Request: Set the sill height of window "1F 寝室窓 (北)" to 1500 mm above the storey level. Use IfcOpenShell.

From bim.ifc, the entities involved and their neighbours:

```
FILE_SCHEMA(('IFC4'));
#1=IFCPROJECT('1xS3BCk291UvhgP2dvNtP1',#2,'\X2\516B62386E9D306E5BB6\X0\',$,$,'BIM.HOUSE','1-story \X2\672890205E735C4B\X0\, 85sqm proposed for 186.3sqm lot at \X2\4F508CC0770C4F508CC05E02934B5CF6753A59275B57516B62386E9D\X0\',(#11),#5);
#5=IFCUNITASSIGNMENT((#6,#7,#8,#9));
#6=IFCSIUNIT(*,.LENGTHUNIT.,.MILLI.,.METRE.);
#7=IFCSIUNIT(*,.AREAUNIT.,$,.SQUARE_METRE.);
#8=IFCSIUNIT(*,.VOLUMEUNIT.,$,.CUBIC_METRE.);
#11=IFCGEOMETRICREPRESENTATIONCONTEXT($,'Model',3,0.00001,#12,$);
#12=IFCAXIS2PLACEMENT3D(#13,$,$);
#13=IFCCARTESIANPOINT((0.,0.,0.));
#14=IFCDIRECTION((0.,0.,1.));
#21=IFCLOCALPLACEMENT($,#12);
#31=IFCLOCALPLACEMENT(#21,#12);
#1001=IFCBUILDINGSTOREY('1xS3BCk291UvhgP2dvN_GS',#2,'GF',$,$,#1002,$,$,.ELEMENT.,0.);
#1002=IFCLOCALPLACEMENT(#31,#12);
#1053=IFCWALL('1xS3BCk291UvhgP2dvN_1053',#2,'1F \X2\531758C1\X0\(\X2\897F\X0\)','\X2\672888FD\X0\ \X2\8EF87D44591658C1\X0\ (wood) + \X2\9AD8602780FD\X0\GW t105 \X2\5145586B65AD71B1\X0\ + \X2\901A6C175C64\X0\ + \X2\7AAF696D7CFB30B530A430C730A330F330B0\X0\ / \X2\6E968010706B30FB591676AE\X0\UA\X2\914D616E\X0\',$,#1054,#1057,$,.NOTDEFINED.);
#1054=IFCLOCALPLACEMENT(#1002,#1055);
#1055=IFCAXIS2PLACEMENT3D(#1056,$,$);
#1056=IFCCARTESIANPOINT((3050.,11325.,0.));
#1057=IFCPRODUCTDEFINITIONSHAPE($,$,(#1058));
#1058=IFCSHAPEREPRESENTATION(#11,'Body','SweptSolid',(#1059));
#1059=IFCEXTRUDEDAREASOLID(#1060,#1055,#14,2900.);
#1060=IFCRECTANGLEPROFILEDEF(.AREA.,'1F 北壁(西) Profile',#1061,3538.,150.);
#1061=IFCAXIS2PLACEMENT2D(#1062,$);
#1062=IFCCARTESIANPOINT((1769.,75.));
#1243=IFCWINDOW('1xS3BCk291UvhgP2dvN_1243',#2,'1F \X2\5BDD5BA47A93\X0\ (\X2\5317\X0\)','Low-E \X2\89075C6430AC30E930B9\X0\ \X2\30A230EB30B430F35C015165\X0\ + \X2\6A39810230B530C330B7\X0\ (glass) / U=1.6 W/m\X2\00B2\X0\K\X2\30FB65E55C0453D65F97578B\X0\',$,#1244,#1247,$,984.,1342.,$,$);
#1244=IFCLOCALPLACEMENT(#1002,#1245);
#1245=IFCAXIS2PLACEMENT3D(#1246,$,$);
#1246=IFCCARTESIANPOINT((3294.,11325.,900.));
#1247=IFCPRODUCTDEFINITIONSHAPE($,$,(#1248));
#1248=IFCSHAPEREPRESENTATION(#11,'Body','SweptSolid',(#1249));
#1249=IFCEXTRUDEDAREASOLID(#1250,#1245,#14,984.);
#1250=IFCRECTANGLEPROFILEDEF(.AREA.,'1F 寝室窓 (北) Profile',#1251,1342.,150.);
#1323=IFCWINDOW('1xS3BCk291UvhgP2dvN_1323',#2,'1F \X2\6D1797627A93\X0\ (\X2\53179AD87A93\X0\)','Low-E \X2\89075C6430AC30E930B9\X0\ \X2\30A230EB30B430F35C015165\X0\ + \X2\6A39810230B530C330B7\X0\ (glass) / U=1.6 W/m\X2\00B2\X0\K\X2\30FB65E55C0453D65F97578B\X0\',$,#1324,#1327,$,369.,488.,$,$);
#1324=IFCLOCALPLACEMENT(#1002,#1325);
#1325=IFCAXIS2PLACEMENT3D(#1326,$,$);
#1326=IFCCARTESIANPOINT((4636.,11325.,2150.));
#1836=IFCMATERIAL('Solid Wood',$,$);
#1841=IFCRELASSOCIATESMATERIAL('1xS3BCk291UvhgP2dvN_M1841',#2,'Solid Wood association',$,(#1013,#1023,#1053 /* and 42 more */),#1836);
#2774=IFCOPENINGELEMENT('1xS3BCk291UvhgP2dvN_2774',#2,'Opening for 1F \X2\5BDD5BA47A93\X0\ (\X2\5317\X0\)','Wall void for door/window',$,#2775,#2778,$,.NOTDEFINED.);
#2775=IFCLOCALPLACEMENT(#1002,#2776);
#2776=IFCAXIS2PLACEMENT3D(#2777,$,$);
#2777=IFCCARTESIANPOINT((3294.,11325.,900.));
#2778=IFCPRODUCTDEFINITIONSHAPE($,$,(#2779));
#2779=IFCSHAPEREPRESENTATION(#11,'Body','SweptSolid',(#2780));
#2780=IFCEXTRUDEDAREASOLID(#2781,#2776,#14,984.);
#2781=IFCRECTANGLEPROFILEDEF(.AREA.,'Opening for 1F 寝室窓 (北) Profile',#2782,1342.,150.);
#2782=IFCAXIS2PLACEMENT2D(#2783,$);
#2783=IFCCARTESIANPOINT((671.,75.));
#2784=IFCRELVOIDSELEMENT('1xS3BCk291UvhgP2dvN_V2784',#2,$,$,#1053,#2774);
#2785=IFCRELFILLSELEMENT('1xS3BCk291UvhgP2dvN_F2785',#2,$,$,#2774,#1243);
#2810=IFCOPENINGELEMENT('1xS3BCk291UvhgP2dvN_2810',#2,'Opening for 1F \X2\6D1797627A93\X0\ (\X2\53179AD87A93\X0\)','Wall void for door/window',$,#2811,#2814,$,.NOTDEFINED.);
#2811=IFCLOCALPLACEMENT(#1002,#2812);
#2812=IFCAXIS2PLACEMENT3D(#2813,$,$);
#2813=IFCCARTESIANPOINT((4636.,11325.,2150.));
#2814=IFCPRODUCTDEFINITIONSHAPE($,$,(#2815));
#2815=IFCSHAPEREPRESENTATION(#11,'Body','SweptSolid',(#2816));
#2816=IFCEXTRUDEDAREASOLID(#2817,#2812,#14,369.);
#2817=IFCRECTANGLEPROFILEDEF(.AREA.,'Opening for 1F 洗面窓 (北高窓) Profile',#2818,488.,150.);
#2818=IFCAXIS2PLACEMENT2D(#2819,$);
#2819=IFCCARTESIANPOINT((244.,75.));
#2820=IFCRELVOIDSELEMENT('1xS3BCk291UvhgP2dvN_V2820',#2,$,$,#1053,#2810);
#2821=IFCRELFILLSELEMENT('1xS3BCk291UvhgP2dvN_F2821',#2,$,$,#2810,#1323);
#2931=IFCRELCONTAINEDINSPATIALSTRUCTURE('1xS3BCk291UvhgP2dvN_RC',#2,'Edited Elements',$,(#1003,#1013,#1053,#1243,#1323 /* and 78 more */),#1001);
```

```python
import numpy as np
import ifcopenshell
import ifcopenshell.api.geometry
import ifcopenshell.geom
import ifcopenshell.util.element
import ifcopenshell.util.placement
import ifcopenshell.util.shape
import ifcopenshell.util.unit

model = ifcopenshell.open("bim.ifc")
unit_scale = ifcopenshell.util.unit.calculate_unit_scale(model)

window = model.by_guid("1xS3BCk291UvhgP2dvN_1243")
opening = window.FillsVoids[0].RelatingOpeningElement
storey = ifcopenshell.util.element.get_container(window, ifc_class="IfcBuildingStorey")
level = ifcopenshell.util.placement.get_local_placement(storey.ObjectPlacement)[2, 3]

# The opening's origin need not be at the sill, so measure its lowest point.
shape = ifcopenshell.geom.create_shape(ifcopenshell.geom.settings(), opening)
bottom = ifcopenshell.util.shape.get_shape_bottom_elevation(shape, shape.geometry) / unit_scale
dz = level + 1.5 / unit_scale - bottom

shift = np.array([0.0, 0.0, dz])
# The window is not placed relative to its opening, so move both.
for product in (opening, window):
    matrix = ifcopenshell.util.placement.get_local_placement(product.ObjectPlacement)
    matrix[:3, 3] += shift
    ifcopenshell.api.geometry.edit_object_placement(model, product=product, matrix=matrix, is_si=False)

print(f"moved by {dz * unit_scale:+.3f} m")

model.write("bim_edited.ifc")
```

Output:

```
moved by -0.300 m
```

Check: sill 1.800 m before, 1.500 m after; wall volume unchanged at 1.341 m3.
